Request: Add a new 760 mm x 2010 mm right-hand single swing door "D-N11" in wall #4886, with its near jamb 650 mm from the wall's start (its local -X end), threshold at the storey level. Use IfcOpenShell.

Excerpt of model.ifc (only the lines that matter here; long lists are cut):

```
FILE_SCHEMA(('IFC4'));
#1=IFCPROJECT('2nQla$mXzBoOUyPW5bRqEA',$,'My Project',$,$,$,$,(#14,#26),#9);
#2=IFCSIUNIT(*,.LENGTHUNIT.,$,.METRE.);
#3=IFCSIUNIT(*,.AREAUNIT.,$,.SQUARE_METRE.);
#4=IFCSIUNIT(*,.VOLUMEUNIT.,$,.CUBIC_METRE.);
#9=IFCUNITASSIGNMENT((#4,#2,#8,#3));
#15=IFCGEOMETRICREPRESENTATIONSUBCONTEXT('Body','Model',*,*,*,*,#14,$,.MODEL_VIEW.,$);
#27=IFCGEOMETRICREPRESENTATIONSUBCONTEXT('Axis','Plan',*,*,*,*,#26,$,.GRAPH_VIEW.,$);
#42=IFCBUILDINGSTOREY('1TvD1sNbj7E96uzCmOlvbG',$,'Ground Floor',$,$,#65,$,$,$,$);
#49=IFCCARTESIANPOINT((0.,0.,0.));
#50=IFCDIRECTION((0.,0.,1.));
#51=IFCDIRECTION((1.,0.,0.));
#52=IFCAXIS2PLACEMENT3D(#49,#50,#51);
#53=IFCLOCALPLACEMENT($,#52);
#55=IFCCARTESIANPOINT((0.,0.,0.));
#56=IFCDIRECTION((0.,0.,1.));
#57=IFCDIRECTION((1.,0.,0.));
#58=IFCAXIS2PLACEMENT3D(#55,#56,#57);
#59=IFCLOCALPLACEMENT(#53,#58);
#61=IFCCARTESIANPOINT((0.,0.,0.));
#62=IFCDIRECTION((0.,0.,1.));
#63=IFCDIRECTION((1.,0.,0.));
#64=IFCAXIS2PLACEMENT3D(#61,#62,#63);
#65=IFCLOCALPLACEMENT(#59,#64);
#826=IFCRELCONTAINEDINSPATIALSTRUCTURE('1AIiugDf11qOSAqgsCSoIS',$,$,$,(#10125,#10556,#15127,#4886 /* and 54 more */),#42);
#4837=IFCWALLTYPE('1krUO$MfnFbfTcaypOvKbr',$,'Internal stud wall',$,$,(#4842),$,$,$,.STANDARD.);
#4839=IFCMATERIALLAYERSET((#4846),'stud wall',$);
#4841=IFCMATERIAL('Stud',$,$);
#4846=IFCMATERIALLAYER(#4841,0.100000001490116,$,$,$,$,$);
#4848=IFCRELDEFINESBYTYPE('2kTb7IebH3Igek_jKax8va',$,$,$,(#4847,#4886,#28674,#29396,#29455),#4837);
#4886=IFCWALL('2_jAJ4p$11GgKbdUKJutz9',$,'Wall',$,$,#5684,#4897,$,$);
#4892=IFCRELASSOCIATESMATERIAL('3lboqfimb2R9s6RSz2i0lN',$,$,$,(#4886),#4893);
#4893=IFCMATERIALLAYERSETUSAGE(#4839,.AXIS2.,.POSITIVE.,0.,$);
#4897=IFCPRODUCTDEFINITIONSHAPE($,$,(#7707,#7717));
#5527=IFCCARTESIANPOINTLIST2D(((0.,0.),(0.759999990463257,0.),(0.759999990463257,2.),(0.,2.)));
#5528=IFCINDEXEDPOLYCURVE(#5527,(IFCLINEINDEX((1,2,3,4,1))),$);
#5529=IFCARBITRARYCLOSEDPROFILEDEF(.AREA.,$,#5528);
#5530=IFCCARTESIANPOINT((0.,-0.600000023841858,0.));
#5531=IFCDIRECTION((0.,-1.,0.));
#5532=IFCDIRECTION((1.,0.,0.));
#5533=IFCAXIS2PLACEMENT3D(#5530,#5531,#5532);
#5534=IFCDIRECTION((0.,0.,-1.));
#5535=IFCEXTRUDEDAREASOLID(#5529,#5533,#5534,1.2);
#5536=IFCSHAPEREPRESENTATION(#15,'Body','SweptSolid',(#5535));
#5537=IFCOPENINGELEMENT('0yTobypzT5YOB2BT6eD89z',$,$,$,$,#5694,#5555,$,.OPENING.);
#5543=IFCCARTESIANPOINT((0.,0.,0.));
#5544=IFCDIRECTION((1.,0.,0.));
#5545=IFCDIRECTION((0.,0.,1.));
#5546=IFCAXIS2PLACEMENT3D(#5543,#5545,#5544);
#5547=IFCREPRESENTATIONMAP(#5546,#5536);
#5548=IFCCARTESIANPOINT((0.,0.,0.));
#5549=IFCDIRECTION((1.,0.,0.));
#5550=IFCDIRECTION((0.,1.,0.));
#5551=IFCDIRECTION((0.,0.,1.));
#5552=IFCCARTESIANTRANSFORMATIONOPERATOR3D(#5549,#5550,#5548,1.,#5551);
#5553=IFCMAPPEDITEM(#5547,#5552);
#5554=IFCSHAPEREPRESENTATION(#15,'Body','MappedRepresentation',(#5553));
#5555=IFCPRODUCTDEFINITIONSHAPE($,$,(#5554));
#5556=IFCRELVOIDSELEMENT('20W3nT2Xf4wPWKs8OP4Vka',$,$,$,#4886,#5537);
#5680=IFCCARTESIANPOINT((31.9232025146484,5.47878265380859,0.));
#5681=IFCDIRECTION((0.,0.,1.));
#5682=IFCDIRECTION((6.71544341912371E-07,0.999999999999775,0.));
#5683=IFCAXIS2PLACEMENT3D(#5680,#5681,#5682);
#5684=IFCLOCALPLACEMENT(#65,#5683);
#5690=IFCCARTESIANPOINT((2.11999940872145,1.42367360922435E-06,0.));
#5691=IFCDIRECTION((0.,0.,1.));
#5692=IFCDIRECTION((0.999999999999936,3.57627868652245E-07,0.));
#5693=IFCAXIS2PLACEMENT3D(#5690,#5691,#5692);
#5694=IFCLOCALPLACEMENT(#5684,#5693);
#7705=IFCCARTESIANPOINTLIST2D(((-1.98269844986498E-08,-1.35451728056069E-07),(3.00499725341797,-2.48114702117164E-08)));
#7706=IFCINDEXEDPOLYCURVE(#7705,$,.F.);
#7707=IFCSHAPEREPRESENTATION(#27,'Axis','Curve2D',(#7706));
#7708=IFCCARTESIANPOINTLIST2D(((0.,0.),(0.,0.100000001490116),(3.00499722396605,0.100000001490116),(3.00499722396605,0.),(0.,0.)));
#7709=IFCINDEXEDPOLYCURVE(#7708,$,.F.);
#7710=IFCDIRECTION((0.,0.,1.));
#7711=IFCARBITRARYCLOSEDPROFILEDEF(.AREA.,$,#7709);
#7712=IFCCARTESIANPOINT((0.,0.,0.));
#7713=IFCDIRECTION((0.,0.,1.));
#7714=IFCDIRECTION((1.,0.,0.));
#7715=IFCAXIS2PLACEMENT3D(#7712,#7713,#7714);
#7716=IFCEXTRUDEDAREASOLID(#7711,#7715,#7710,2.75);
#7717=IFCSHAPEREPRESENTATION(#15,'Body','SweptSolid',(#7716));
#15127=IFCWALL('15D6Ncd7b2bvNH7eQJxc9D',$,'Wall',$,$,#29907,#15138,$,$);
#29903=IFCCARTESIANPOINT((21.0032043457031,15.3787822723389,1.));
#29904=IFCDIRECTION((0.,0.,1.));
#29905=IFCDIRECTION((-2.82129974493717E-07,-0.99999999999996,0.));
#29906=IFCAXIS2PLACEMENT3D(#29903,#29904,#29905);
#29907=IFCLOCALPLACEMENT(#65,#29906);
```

```python
import numpy as np
import ifcopenshell
import ifcopenshell.api.feature
import ifcopenshell.api.geometry
import ifcopenshell.api.root
import ifcopenshell.api.spatial
import ifcopenshell.geom
import ifcopenshell.util.element
import ifcopenshell.util.placement
import ifcopenshell.util.representation
import ifcopenshell.util.shape
import ifcopenshell.util.unit

model = ifcopenshell.open("model.ifc")
unit_scale = ifcopenshell.util.unit.calculate_unit_scale(model)
settings = ifcopenshell.geom.settings()


def volume(element):
    """Net volume in cubic metres, openings subtracted."""
    shape = ifcopenshell.geom.create_shape(settings, element)
    return ifcopenshell.util.shape.get_volume(shape.geometry)


wall = model.by_guid("2_jAJ4p$11GgKbdUKJutz9")
storey = ifcopenshell.util.element.get_container(wall, ifc_class="IfcBuildingStorey")
context = ifcopenshell.util.representation.get_context(model, "Model", "Body", "MODEL_VIEW")
before = volume(wall)

width, height, from_end, sill = 0.76, 2.01, 0.65, 0.0  # metres

# The wall runs along its own X axis, and the end named is its -X end.
wall_shape = ifcopenshell.geom.create_shape(settings, wall)
x, y, z = ifcopenshell.util.shape.get_vertices(wall_shape.geometry).T
start = x.min() + from_end
face, thickness = float(y.min()), float(y.max() - y.min())
wall_matrix = ifcopenshell.util.placement.get_local_placement(wall.ObjectPlacement)
level = ifcopenshell.util.placement.get_local_placement(storey.ObjectPlacement)[2, 3]


def in_wall(x, y):
    """Placement at x, y metres in the wall's axes, at sill height."""
    matrix = wall_matrix.copy()
    matrix[:, 3] = wall_matrix @ np.array([x / unit_scale, y / unit_scale, 0.0, 1.0])
    matrix[2, 3] = level + sill / unit_scale
    return matrix


# Opening: a box that overshoots both wall faces by 50 mm.
opening = ifcopenshell.api.root.create_entity(model, ifc_class="IfcOpeningElement", predefined_type="OPENING")
box = ifcopenshell.api.geometry.add_wall_representation(
    model, context=context, length=width, height=height, thickness=thickness + 0.1
)
ifcopenshell.api.geometry.assign_representation(model, product=opening, representation=box)
ifcopenshell.api.geometry.edit_object_placement(model, product=opening, matrix=in_wall(start, face - 0.05), is_si=False)
ifcopenshell.api.feature.add_feature(model, feature=opening, element=wall)

door = ifcopenshell.api.root.create_entity(model, ifc_class="IfcDoor", name="D-N11", predefined_type="DOOR")
door.OverallWidth, door.OverallHeight = width / unit_scale, height / unit_scale
door.OperationType = "SINGLE_SWING_RIGHT"
body = ifcopenshell.api.geometry.add_door_representation(
    model,
    context=context,
    overall_width=door.OverallWidth,
    overall_height=door.OverallHeight,
    operation_type="SINGLE_SWING_RIGHT",
    lining_properties={"LiningDepth": thickness / unit_scale, "ThresholdDepth": thickness / unit_scale},
)
ifcopenshell.api.geometry.assign_representation(model, product=door, representation=body)
ifcopenshell.api.spatial.assign_container(model, products=[door], relating_structure=storey)
ifcopenshell.api.feature.add_filling(model, opening=opening, element=door)

# The lining spans the wall, so the door starts at the wall face.
ifcopenshell.api.geometry.edit_object_placement(model, product=door, matrix=in_wall(start, face), is_si=False)

after = volume(wall)

print(f"wall volume {before:.3f} -> {after:.3f} m3")

model.write("model_v2.ifc")
```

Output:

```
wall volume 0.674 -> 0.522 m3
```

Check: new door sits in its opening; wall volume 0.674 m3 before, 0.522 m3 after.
